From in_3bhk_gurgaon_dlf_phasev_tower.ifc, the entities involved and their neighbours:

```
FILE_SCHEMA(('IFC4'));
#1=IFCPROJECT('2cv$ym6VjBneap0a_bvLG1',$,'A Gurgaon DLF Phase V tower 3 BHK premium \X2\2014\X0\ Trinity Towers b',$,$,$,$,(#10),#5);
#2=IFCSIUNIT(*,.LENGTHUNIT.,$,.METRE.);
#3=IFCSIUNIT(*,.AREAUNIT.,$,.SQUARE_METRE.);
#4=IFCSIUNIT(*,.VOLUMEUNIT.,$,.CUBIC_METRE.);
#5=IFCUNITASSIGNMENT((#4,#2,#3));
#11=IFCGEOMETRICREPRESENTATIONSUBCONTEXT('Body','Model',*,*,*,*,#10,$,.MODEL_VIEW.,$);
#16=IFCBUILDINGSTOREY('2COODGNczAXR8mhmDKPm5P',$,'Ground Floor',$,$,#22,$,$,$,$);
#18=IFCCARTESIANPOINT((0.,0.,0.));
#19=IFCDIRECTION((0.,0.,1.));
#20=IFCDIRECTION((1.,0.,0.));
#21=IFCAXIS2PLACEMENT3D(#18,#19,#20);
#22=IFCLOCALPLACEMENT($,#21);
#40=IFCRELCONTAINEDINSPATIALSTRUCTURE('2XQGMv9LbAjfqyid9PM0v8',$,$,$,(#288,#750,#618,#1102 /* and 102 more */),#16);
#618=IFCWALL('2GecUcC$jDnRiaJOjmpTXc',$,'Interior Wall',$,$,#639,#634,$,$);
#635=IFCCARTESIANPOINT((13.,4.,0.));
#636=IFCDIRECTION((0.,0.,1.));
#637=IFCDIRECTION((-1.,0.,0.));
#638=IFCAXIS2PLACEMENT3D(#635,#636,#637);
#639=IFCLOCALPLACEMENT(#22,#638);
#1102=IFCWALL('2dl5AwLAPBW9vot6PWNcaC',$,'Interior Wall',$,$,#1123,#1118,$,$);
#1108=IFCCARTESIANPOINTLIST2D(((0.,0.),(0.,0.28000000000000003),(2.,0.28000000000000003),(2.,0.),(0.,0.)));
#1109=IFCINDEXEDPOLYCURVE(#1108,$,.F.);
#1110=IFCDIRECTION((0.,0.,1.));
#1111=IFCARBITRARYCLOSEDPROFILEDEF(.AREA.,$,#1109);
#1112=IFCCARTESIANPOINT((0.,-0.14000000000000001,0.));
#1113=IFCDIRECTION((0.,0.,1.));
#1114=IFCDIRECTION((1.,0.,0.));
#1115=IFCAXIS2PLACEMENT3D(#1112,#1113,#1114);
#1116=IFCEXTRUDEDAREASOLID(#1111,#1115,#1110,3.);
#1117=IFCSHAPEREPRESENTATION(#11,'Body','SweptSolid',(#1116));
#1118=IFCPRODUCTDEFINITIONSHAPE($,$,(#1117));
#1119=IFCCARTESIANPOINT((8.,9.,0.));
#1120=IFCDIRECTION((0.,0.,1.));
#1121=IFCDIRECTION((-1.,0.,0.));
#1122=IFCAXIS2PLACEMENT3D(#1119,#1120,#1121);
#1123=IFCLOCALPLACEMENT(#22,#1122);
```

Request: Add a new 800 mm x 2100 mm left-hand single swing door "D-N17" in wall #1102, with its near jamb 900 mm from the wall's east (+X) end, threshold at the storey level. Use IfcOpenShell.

```python
import numpy as np
import ifcopenshell
import ifcopenshell.api.feature
import ifcopenshell.api.geometry
import ifcopenshell.api.root
import ifcopenshell.api.spatial
import ifcopenshell.geom
import ifcopenshell.util.element
import ifcopenshell.util.placement
import ifcopenshell.util.representation
import ifcopenshell.util.shape
import ifcopenshell.util.unit

model = ifcopenshell.open("in_3bhk_gurgaon_dlf_phasev_tower.ifc")
unit_scale = ifcopenshell.util.unit.calculate_unit_scale(model)
settings = ifcopenshell.geom.settings()


def volume(element):
    """Net volume in cubic metres, openings subtracted."""
    shape = ifcopenshell.geom.create_shape(settings, element)
    return ifcopenshell.util.shape.get_volume(shape.geometry)


wall = model.by_guid("2dl5AwLAPBW9vot6PWNcaC")
storey = ifcopenshell.util.element.get_container(wall, ifc_class="IfcBuildingStorey")
context = ifcopenshell.util.representation.get_context(model, "Model", "Body", "MODEL_VIEW")
before = volume(wall)

width, height, from_end, sill = 0.8, 2.1, 0.9, 0.0  # metres

# The wall runs along its own X axis, and the end named is its -X end.
wall_shape = ifcopenshell.geom.create_shape(settings, wall)
x, y, z = ifcopenshell.util.shape.get_vertices(wall_shape.geometry).T
start = x.min() + from_end
face, thickness = float(y.min()), float(y.max() - y.min())
wall_matrix = ifcopenshell.util.placement.get_local_placement(wall.ObjectPlacement)
level = ifcopenshell.util.placement.get_local_placement(storey.ObjectPlacement)[2, 3]


def in_wall(x, y):
    """Placement at x, y metres in the wall's axes, at sill height."""
    matrix = wall_matrix.copy()
    matrix[:, 3] = wall_matrix @ np.array([x / unit_scale, y / unit_scale, 0.0, 1.0])
    matrix[2, 3] = level + sill / unit_scale
    return matrix


# Opening: a box that overshoots both wall faces by 50 mm.
opening = ifcopenshell.api.root.create_entity(model, ifc_class="IfcOpeningElement", predefined_type="OPENING")
box = ifcopenshell.api.geometry.add_wall_representation(
    model, context=context, length=width, height=height, thickness=thickness + 0.1
)
ifcopenshell.api.geometry.assign_representation(model, product=opening, representation=box)
ifcopenshell.api.geometry.edit_object_placement(model, product=opening, matrix=in_wall(start, face - 0.05), is_si=False)
ifcopenshell.api.feature.add_feature(model, feature=opening, element=wall)

door = ifcopenshell.api.root.create_entity(model, ifc_class="IfcDoor", name="D-N17", predefined_type="DOOR")
door.OverallWidth, door.OverallHeight = width / unit_scale, height / unit_scale
door.OperationType = "SINGLE_SWING_LEFT"
body = ifcopenshell.api.geometry.add_door_representation(
    model,
    context=context,
    overall_width=door.OverallWidth,
    overall_height=door.OverallHeight,
    operation_type="SINGLE_SWING_LEFT",
    lining_properties={"LiningDepth": thickness / unit_scale, "ThresholdDepth": thickness / unit_scale},
)
ifcopenshell.api.geometry.assign_representation(model, product=door, representation=body)
ifcopenshell.api.spatial.assign_container(model, products=[door], relating_structure=storey)
ifcopenshell.api.feature.add_filling(model, opening=opening, element=door)

# The lining spans the wall, so the door starts at the wall face.
ifcopenshell.api.geometry.edit_object_placement(model, product=door, matrix=in_wall(start, face), is_si=False)

after = volume(wall)

print(f"wall volume {before:.3f} -> {after:.3f} m3")

model.write("in_3bhk_gurgaon_dlf_phasev_tower-out.ifc")
```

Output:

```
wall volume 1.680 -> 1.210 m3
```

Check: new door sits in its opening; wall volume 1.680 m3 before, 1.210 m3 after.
